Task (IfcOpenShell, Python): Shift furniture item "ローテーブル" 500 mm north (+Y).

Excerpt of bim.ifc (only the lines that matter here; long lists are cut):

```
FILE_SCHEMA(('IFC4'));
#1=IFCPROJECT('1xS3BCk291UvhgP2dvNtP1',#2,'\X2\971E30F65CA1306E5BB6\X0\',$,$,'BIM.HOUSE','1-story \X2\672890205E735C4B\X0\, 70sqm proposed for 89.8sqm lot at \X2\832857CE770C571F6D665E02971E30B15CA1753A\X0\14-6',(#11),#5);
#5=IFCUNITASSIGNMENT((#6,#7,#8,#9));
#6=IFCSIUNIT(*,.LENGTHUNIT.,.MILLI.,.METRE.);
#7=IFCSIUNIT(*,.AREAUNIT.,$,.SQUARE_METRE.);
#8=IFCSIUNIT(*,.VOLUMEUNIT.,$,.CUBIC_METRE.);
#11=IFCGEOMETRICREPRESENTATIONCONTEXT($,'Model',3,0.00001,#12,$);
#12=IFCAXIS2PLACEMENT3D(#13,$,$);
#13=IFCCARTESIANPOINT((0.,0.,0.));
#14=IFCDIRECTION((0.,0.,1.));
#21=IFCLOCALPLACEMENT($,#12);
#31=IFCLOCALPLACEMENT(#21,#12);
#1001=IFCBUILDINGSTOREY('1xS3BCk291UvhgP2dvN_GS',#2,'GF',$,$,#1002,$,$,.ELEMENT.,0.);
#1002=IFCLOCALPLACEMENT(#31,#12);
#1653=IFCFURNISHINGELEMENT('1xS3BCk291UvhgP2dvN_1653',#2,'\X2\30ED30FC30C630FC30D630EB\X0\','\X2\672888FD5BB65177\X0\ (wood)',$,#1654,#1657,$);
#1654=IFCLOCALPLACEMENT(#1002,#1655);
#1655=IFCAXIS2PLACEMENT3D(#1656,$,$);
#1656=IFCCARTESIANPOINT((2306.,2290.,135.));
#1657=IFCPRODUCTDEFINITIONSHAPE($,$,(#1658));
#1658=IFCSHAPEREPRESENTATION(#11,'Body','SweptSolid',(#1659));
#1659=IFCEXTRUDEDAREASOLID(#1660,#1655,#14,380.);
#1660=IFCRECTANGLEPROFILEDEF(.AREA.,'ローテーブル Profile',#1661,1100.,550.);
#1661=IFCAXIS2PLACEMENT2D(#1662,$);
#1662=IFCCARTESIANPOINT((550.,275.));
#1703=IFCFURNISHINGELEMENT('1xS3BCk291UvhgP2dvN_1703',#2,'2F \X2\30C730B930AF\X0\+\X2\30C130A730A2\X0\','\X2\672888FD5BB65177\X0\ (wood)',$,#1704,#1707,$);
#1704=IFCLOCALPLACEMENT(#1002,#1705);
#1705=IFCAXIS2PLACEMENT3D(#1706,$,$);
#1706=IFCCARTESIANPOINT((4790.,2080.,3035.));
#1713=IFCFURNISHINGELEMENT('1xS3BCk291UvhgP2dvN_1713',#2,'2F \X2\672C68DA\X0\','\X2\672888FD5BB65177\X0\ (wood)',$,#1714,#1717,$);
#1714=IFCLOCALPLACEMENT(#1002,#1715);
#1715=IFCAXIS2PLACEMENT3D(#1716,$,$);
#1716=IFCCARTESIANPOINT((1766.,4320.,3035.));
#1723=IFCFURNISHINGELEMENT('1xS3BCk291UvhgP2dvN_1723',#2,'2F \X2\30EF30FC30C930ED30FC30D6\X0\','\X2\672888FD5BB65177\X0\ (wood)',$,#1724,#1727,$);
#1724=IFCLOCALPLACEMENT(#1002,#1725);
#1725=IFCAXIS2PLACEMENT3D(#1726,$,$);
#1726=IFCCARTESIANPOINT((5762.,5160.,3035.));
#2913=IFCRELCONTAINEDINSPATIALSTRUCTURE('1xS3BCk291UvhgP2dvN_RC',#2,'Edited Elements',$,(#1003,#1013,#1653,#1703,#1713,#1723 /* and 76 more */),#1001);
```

```python
import ifcopenshell
import ifcopenshell.api.geometry
import ifcopenshell.util.placement
import ifcopenshell.util.unit

model = ifcopenshell.open("bim.ifc")
unit_scale = ifcopenshell.util.unit.calculate_unit_scale(model)

item = model.by_id(1653)
matrix = ifcopenshell.util.placement.get_local_placement(item.ObjectPlacement)
matrix[1, 3] += 0.5 / unit_scale
ifcopenshell.api.geometry.edit_object_placement(model, product=item, matrix=matrix, is_si=False)

print(ifcopenshell.util.placement.get_local_placement(item.ObjectPlacement).round(3) + 0.0)

model.write("bim_v2.ifc")
```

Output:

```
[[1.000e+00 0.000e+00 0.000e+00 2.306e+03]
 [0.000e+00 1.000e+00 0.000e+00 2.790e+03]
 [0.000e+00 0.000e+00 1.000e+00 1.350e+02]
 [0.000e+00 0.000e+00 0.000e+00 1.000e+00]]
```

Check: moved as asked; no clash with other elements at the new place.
